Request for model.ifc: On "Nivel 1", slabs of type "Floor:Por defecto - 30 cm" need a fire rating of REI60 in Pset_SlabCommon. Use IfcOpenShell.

First a look at what the model holds.

```python
import ifcopenshell
import ifcopenshell.util.element

model = ifcopenshell.open("model.ifc")
print(model.schema)
storey = next(s for s in model.by_type("IfcBuildingStorey") if s.Name == "Nivel 1")
slabs = [e for e in ifcopenshell.util.element.get_decomposition(storey) if e.is_a("IfcSlab")]
seen = {}
for e in slabs:
    element_type = ifcopenshell.util.element.get_type(e)
    key = (element_type.Name if element_type != e and element_type else None, ifcopenshell.util.element.get_pset(e, "Pset_SlabCommon", "FireRating"))
    seen[key] = seen.get(key, 0) + 1
for (name, value), count in sorted(seen.items(), key=str):
    print(count, "x", name, "|", value)
```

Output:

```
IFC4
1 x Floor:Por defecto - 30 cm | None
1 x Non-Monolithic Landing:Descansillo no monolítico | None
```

```python
import ifcopenshell
import ifcopenshell.api.pset
import ifcopenshell.util.element

model = ifcopenshell.open("model.ifc")

storey = next(s for s in model.by_type("IfcBuildingStorey") if s.Name == "Nivel 1")
slabs = [e for e in ifcopenshell.util.element.get_decomposition(storey) if e.is_a("IfcSlab")]

count = 0
for e in slabs:
    element_type = ifcopenshell.util.element.get_type(e)
    if element_type in (None, e) or element_type.Name != "Floor:Por defecto - 30 cm":
        continue
    # add_pset returns the element's existing set when there is one.
    pset = ifcopenshell.api.pset.add_pset(model, product=e, name="Pset_SlabCommon")
    ifcopenshell.api.pset.edit_pset(model, pset=pset, properties={"FireRating": "REI60"})
    count += 1

print(count, "slabs updated")

model.write("model_rev.ifc")
```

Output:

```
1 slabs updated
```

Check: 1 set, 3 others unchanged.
